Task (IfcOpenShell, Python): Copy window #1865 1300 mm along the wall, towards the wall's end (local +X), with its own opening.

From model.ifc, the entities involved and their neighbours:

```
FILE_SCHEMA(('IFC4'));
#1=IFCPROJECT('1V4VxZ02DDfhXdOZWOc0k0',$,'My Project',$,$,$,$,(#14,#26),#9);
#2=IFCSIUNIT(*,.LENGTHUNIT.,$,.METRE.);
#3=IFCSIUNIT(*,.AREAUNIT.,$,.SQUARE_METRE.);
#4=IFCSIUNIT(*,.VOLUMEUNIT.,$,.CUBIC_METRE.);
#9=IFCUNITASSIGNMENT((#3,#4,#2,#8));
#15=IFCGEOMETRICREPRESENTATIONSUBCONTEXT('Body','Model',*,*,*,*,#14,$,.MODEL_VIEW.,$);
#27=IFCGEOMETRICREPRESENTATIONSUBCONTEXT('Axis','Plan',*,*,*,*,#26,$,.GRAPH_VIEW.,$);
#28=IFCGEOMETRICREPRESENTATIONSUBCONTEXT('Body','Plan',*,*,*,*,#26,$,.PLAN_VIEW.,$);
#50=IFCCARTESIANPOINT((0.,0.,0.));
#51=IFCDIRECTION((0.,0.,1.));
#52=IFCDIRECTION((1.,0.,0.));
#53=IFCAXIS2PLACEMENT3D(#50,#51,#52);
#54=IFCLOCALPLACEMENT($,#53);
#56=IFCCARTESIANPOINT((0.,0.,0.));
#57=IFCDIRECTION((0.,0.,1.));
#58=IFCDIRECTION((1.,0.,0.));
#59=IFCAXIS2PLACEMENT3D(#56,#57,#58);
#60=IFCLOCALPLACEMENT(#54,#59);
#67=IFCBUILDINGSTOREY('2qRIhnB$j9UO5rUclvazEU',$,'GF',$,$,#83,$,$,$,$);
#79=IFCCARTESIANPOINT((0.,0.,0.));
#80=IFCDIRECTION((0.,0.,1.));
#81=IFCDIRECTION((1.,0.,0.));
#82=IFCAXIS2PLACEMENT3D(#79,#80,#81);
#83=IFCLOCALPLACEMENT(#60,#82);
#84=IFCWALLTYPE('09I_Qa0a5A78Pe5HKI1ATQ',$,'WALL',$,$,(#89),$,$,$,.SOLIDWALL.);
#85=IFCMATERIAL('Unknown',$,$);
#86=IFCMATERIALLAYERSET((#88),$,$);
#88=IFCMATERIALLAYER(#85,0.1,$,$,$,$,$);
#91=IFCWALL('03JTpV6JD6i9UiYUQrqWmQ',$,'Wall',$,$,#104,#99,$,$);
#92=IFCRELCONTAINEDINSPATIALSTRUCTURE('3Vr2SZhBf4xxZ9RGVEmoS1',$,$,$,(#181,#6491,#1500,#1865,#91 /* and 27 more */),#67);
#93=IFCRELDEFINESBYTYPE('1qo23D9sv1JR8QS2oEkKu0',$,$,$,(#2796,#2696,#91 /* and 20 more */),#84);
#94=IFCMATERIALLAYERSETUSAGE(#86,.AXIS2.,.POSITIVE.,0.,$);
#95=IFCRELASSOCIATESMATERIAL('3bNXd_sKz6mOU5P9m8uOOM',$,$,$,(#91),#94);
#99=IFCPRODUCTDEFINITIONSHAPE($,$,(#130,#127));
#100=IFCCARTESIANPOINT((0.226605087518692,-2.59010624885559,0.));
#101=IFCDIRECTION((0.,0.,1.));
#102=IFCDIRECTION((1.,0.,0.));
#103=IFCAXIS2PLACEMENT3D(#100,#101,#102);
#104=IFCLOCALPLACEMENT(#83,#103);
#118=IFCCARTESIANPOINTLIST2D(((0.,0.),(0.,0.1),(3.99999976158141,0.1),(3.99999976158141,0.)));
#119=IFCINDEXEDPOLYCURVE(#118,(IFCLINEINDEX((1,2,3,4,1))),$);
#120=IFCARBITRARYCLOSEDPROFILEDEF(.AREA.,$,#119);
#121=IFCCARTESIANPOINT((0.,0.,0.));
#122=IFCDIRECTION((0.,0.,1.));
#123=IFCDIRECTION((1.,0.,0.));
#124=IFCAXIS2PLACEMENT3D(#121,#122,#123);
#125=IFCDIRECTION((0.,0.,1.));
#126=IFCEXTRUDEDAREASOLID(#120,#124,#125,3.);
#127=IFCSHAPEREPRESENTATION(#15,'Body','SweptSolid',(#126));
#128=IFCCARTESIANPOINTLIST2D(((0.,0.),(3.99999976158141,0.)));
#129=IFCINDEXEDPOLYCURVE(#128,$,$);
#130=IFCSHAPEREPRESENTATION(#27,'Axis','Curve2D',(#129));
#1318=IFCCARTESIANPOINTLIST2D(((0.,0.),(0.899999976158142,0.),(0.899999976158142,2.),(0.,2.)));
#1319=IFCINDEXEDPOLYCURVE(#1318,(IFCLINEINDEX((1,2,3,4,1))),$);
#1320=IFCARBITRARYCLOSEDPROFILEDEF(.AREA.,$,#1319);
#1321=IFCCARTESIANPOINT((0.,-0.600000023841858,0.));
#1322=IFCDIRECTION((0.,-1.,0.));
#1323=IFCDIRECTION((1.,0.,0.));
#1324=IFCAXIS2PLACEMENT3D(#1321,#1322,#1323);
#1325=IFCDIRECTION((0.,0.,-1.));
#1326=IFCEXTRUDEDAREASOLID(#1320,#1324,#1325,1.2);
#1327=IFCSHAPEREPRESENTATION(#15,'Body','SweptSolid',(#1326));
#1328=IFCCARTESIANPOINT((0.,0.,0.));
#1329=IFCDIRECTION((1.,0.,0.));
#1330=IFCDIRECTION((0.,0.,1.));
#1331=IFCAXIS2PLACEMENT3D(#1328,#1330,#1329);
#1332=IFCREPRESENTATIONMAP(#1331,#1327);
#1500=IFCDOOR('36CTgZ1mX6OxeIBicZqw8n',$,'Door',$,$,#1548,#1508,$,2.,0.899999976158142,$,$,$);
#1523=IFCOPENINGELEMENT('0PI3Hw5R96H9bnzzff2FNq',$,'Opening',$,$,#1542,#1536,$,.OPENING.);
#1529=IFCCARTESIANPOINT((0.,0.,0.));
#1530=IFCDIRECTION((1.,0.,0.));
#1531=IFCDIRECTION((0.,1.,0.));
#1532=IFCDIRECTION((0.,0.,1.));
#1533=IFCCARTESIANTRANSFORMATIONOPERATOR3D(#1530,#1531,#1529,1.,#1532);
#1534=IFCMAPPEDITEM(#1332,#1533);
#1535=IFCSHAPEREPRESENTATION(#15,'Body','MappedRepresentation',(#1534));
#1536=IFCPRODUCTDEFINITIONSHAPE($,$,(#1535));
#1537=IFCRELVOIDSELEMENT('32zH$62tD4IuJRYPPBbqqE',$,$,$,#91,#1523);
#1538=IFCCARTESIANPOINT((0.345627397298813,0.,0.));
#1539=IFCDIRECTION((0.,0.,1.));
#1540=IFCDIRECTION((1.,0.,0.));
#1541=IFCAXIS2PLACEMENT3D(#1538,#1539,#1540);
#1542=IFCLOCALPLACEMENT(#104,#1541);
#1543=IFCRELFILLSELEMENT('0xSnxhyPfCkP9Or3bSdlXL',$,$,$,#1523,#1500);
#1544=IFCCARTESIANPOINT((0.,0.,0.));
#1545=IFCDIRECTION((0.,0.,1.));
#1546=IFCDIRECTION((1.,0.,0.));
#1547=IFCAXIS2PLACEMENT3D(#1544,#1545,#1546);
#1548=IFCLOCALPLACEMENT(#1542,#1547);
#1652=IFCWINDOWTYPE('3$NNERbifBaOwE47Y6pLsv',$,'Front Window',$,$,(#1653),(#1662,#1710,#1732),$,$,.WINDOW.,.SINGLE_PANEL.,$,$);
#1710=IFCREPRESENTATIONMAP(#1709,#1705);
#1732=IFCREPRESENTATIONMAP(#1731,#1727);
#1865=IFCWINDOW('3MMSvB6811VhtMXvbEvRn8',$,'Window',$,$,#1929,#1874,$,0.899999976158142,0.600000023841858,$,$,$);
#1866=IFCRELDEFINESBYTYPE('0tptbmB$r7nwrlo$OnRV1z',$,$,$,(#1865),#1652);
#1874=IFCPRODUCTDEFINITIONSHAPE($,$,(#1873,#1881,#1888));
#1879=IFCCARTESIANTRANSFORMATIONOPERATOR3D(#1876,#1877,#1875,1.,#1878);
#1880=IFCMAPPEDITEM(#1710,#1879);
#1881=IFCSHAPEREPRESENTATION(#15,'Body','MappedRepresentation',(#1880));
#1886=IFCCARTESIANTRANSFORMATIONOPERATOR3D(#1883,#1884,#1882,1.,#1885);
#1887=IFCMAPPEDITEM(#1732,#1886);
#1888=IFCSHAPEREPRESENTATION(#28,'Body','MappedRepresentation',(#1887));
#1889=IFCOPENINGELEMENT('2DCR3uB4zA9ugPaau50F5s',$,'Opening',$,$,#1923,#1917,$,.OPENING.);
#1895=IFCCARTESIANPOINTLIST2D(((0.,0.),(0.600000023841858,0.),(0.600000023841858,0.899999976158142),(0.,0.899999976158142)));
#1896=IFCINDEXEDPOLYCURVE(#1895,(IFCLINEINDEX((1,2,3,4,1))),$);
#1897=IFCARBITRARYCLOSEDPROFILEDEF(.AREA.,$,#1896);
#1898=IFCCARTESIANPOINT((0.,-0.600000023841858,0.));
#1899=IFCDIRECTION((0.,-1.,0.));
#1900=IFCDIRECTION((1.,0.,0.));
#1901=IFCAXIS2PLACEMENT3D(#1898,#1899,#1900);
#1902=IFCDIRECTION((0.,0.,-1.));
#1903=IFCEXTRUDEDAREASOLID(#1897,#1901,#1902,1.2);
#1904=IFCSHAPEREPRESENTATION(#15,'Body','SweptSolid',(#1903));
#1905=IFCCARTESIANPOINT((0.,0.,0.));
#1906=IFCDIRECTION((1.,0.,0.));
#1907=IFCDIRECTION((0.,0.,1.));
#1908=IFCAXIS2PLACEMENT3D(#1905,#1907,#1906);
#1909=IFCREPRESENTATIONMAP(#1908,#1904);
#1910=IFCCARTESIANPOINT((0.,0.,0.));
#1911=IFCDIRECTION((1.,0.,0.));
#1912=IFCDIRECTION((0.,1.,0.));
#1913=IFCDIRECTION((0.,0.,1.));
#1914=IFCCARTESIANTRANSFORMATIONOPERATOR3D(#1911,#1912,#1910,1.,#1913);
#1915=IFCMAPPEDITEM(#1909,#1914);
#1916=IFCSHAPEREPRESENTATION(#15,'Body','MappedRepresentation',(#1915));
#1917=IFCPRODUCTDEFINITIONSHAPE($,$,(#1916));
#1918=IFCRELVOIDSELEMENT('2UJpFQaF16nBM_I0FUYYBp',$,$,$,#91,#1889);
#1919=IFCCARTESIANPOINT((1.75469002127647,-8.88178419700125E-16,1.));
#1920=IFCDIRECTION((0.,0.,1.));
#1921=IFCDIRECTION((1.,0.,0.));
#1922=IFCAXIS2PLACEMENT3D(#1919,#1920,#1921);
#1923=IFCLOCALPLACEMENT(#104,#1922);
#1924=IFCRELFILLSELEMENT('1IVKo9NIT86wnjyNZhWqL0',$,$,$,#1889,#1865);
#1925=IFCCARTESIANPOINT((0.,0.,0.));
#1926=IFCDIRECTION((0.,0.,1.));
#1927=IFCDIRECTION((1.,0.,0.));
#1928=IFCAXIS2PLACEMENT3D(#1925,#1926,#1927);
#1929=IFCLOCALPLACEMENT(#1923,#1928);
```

```python
import ifcopenshell
import ifcopenshell.api.feature
import ifcopenshell.api.geometry
import ifcopenshell.api.root
import ifcopenshell.geom
import ifcopenshell.util.element
import ifcopenshell.util.placement
import ifcopenshell.util.shape
import ifcopenshell.util.unit

model = ifcopenshell.open("model.ifc")
unit_scale = ifcopenshell.util.unit.calculate_unit_scale(model)
settings = ifcopenshell.geom.settings()


def volume(element):
    """Net volume in cubic metres, openings subtracted."""
    shape = ifcopenshell.geom.create_shape(settings, element)
    return ifcopenshell.util.shape.get_volume(shape.geometry)


window = model.by_guid("3MMSvB6811VhtMXvbEvRn8")
opening = window.FillsVoids[0].RelatingOpeningElement
wall = opening.VoidsElements[0].RelatingBuildingElement
before = volume(wall)
shift = ifcopenshell.util.placement.get_local_placement(wall.ObjectPlacement)[:3, 0] * 1.3 / unit_scale

# copy_class copies the void relationship, type, container and properties, but no geometry.
new_opening = ifcopenshell.api.root.copy_class(model, product=opening)
new_opening.Representation = ifcopenshell.util.element.copy_deep(
    model, opening.Representation, exclude=["IfcGeometricRepresentationContext", "IfcRepresentationMap"]
)
new_window = ifcopenshell.api.root.copy_class(model, product=window)
new_window.Representation = ifcopenshell.util.element.copy_deep(
    model, window.Representation, exclude=["IfcGeometricRepresentationContext", "IfcRepresentationMap"]
)
ifcopenshell.api.feature.add_filling(model, opening=new_opening, element=new_window)

for old, new in ((opening, new_opening), (window, new_window)):
    matrix = ifcopenshell.util.placement.get_local_placement(old.ObjectPlacement)
    matrix[:3, 3] += shift
    ifcopenshell.api.geometry.edit_object_placement(model, product=new, matrix=matrix, is_si=False)

after = volume(wall)

print(f"wall volume {before:.3f} -> {after:.3f} m3")

model.write("model_rev.ifc")
```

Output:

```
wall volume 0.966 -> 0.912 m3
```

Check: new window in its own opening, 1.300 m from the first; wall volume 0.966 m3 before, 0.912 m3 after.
